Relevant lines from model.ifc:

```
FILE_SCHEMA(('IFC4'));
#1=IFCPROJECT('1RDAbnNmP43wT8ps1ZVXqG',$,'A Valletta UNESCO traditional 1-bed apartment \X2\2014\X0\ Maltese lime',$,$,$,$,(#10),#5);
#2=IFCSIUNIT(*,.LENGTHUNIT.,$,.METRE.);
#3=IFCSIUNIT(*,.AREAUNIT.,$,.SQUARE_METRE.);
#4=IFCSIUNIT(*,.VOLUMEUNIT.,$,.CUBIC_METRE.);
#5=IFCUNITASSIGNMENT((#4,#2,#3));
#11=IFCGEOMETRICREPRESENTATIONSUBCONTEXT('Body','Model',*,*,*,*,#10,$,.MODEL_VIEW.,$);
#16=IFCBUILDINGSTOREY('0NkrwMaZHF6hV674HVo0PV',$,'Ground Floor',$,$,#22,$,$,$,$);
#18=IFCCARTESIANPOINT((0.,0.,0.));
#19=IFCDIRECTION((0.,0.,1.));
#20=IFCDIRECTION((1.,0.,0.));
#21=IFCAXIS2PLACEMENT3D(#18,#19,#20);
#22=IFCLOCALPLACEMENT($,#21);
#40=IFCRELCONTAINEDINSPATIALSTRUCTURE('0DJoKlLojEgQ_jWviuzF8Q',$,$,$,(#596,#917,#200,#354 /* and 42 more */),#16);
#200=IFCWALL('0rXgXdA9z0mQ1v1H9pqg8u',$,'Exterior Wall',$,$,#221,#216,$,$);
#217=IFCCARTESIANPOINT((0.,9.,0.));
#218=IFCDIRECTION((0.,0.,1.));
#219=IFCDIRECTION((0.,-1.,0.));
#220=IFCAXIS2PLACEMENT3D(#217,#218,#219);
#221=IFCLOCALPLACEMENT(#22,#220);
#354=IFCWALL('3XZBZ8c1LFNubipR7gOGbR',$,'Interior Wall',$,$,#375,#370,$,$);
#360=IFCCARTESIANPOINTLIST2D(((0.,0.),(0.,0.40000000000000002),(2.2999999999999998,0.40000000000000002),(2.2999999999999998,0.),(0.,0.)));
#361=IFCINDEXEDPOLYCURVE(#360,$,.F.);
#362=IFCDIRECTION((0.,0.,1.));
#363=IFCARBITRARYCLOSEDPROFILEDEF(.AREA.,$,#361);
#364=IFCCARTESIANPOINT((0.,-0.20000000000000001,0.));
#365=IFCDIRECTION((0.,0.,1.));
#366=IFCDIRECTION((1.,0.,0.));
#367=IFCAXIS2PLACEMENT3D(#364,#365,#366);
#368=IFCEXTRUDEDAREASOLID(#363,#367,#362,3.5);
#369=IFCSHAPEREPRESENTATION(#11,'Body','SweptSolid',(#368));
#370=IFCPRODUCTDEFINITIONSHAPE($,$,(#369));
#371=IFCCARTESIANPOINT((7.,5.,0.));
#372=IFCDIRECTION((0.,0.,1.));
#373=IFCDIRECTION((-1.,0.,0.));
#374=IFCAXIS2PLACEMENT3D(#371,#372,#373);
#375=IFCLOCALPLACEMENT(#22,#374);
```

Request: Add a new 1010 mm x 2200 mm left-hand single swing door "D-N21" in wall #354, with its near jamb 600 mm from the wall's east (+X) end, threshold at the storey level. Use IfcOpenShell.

```python
import numpy as np
import ifcopenshell
import ifcopenshell.api.feature
import ifcopenshell.api.geometry
import ifcopenshell.api.root
import ifcopenshell.api.spatial
import ifcopenshell.geom
import ifcopenshell.util.element
import ifcopenshell.util.placement
import ifcopenshell.util.representation
import ifcopenshell.util.shape
import ifcopenshell.util.unit

model = ifcopenshell.open("model.ifc")
unit_scale = ifcopenshell.util.unit.calculate_unit_scale(model)
settings = ifcopenshell.geom.settings()


def volume(element):
    """Net volume in cubic metres, openings subtracted."""
    shape = ifcopenshell.geom.create_shape(settings, element)
    return ifcopenshell.util.shape.get_volume(shape.geometry)


wall = model.by_guid("3XZBZ8c1LFNubipR7gOGbR")
storey = ifcopenshell.util.element.get_container(wall, ifc_class="IfcBuildingStorey")
context = ifcopenshell.util.representation.get_context(model, "Model", "Body", "MODEL_VIEW")
before = volume(wall)

width, height, from_end, sill = 1.01, 2.2, 0.6, 0.0  # metres

# The wall runs along its own X axis, and the end named is its -X end.
wall_shape = ifcopenshell.geom.create_shape(settings, wall)
x, y, z = ifcopenshell.util.shape.get_vertices(wall_shape.geometry).T
start = x.min() + from_end
face, thickness = float(y.min()), float(y.max() - y.min())
wall_matrix = ifcopenshell.util.placement.get_local_placement(wall.ObjectPlacement)
level = ifcopenshell.util.placement.get_local_placement(storey.ObjectPlacement)[2, 3]


def in_wall(x, y):
    """Placement at x, y metres in the wall's axes, at sill height."""
    matrix = wall_matrix.copy()
    matrix[:, 3] = wall_matrix @ np.array([x / unit_scale, y / unit_scale, 0.0, 1.0])
    matrix[2, 3] = level + sill / unit_scale
    return matrix


# Opening: a box that overshoots both wall faces by 50 mm.
opening = ifcopenshell.api.root.create_entity(model, ifc_class="IfcOpeningElement", predefined_type="OPENING")
box = ifcopenshell.api.geometry.add_wall_representation(
    model, context=context, length=width, height=height, thickness=thickness + 0.1
)
ifcopenshell.api.geometry.assign_representation(model, product=opening, representation=box)
ifcopenshell.api.geometry.edit_object_placement(model, product=opening, matrix=in_wall(start, face - 0.05), is_si=False)
ifcopenshell.api.feature.add_feature(model, feature=opening, element=wall)

door = ifcopenshell.api.root.create_entity(model, ifc_class="IfcDoor", name="D-N21", predefined_type="DOOR")
door.OverallWidth, door.OverallHeight = width / unit_scale, height / unit_scale
door.OperationType = "SINGLE_SWING_LEFT"
body = ifcopenshell.api.geometry.add_door_representation(
    model,
    context=context,
    overall_width=door.OverallWidth,
    overall_height=door.OverallHeight,
    operation_type="SINGLE_SWING_LEFT",
    lining_properties={"LiningDepth": thickness / unit_scale, "ThresholdDepth": thickness / unit_scale},
)
ifcopenshell.api.geometry.assign_representation(model, product=door, representation=body)
ifcopenshell.api.spatial.assign_container(model, products=[door], relating_structure=storey)
ifcopenshell.api.feature.add_filling(model, opening=opening, element=door)

# The lining spans the wall, so the door starts at the wall face.
ifcopenshell.api.geometry.edit_object_placement(model, product=door, matrix=in_wall(start, face), is_si=False)

after = volume(wall)

print(f"wall volume {before:.3f} -> {after:.3f} m3")

model.write("model_edited.ifc")
```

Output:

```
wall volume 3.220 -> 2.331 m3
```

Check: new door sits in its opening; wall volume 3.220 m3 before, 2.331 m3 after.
